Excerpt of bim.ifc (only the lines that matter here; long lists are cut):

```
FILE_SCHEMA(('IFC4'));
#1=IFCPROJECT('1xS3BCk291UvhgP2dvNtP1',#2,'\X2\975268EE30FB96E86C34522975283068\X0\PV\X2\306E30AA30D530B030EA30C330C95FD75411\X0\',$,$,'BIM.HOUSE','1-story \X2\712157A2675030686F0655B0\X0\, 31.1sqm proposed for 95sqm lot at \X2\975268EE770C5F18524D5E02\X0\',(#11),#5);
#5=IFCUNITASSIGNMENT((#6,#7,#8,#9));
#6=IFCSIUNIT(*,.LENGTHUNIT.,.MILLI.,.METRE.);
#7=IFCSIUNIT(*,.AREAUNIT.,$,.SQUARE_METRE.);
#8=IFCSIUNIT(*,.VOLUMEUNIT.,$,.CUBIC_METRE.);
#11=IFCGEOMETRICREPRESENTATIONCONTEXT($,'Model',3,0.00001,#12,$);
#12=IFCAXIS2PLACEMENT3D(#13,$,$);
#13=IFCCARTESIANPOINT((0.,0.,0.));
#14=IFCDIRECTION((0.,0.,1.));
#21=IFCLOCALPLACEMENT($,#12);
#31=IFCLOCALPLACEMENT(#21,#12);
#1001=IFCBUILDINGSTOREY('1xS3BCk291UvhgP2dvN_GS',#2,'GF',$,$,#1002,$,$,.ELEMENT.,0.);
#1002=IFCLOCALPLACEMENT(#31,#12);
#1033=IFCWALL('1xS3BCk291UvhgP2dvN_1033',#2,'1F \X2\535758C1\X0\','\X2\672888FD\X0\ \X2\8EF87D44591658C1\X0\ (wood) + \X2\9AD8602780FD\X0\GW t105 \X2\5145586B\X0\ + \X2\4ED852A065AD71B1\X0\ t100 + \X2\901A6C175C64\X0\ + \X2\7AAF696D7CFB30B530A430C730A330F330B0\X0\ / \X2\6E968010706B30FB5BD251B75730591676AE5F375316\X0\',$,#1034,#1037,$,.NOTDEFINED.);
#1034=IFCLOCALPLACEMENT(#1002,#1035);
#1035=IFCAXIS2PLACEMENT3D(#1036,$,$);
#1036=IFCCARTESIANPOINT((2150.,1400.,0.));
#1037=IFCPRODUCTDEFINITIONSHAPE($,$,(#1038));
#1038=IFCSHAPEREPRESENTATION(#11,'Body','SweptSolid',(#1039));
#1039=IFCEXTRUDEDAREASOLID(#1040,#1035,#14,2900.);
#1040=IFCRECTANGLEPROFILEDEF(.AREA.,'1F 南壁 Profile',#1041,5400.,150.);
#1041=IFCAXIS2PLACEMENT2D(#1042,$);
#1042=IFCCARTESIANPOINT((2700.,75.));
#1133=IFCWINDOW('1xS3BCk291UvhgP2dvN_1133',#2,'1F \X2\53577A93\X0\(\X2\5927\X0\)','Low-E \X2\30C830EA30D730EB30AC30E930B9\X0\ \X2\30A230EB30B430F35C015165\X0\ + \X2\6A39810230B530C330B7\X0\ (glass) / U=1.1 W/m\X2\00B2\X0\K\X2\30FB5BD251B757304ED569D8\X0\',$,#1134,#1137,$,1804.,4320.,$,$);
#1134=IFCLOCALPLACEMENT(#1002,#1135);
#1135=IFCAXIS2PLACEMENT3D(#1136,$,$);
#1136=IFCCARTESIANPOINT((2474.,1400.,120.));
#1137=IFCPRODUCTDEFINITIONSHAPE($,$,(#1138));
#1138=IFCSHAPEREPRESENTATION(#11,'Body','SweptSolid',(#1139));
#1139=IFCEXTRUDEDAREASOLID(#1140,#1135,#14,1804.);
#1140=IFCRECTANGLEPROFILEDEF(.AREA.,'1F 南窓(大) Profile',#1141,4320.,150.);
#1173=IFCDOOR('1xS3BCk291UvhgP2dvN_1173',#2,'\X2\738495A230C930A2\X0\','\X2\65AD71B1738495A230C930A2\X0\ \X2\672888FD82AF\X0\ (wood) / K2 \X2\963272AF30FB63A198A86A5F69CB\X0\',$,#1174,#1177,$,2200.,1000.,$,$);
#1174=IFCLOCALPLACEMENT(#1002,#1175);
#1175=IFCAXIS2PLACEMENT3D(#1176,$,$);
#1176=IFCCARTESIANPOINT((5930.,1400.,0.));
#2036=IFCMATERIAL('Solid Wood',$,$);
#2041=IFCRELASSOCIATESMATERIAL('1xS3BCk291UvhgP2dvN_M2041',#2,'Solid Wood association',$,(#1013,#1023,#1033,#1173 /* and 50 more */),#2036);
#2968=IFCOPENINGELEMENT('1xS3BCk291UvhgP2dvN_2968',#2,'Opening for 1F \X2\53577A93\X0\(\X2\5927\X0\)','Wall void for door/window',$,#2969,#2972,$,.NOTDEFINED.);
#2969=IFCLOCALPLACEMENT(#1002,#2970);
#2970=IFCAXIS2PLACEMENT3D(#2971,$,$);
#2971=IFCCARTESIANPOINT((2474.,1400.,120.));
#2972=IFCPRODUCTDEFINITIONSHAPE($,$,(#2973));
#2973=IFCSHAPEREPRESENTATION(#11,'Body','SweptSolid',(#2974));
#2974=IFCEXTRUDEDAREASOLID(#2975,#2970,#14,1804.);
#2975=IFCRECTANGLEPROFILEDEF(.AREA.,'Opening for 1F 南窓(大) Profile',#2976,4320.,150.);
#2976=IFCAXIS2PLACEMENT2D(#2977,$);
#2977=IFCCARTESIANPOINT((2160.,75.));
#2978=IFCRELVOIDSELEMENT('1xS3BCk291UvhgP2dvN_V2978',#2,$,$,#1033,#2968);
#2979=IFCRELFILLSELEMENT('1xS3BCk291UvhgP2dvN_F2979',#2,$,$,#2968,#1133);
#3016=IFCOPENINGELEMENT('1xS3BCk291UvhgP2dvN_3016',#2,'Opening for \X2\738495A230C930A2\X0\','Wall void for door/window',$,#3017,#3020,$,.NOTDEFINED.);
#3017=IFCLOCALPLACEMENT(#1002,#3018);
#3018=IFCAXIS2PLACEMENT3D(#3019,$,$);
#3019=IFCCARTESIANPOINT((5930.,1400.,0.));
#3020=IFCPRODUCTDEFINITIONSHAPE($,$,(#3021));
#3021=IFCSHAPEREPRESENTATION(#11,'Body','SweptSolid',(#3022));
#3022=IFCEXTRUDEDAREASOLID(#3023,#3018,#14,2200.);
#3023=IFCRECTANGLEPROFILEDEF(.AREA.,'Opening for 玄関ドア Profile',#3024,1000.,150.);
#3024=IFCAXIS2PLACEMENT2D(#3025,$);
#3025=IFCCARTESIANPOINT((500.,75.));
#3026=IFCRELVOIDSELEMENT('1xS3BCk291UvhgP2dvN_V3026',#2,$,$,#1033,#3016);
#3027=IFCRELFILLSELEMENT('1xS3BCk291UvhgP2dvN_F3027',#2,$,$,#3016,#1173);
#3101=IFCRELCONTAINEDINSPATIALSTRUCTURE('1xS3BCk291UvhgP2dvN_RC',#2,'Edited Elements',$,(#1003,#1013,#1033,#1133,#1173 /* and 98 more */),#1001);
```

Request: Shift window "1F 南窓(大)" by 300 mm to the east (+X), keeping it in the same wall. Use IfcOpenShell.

```python
import ifcopenshell
import ifcopenshell.api.geometry
import ifcopenshell.util.placement

model = ifcopenshell.open("bim.ifc")

window = model.by_guid("1xS3BCk291UvhgP2dvN_1133")
opening = window.FillsVoids[0].RelatingOpeningElement
wall = opening.VoidsElements[0].RelatingBuildingElement

wall_matrix = ifcopenshell.util.placement.get_local_placement(wall.ObjectPlacement)
shift = wall_matrix[:3, 0] * 300.0
before = ifcopenshell.util.placement.get_local_placement(window.ObjectPlacement)[:3, 3].copy()

# The window is not placed relative to its opening, so move both.
for product in (opening, window):
    matrix = ifcopenshell.util.placement.get_local_placement(product.ObjectPlacement)
    matrix[:3, 3] += shift
    ifcopenshell.api.geometry.edit_object_placement(model, product=product, matrix=matrix, is_si=False)

after = ifcopenshell.util.placement.get_local_placement(window.ObjectPlacement)[:3, 3]
print("window moved by", (after - before).round(3) + 0.0)

model.write("bim_updated.ifc")
```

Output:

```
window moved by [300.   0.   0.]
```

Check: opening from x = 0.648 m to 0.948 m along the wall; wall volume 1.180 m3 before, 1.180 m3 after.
